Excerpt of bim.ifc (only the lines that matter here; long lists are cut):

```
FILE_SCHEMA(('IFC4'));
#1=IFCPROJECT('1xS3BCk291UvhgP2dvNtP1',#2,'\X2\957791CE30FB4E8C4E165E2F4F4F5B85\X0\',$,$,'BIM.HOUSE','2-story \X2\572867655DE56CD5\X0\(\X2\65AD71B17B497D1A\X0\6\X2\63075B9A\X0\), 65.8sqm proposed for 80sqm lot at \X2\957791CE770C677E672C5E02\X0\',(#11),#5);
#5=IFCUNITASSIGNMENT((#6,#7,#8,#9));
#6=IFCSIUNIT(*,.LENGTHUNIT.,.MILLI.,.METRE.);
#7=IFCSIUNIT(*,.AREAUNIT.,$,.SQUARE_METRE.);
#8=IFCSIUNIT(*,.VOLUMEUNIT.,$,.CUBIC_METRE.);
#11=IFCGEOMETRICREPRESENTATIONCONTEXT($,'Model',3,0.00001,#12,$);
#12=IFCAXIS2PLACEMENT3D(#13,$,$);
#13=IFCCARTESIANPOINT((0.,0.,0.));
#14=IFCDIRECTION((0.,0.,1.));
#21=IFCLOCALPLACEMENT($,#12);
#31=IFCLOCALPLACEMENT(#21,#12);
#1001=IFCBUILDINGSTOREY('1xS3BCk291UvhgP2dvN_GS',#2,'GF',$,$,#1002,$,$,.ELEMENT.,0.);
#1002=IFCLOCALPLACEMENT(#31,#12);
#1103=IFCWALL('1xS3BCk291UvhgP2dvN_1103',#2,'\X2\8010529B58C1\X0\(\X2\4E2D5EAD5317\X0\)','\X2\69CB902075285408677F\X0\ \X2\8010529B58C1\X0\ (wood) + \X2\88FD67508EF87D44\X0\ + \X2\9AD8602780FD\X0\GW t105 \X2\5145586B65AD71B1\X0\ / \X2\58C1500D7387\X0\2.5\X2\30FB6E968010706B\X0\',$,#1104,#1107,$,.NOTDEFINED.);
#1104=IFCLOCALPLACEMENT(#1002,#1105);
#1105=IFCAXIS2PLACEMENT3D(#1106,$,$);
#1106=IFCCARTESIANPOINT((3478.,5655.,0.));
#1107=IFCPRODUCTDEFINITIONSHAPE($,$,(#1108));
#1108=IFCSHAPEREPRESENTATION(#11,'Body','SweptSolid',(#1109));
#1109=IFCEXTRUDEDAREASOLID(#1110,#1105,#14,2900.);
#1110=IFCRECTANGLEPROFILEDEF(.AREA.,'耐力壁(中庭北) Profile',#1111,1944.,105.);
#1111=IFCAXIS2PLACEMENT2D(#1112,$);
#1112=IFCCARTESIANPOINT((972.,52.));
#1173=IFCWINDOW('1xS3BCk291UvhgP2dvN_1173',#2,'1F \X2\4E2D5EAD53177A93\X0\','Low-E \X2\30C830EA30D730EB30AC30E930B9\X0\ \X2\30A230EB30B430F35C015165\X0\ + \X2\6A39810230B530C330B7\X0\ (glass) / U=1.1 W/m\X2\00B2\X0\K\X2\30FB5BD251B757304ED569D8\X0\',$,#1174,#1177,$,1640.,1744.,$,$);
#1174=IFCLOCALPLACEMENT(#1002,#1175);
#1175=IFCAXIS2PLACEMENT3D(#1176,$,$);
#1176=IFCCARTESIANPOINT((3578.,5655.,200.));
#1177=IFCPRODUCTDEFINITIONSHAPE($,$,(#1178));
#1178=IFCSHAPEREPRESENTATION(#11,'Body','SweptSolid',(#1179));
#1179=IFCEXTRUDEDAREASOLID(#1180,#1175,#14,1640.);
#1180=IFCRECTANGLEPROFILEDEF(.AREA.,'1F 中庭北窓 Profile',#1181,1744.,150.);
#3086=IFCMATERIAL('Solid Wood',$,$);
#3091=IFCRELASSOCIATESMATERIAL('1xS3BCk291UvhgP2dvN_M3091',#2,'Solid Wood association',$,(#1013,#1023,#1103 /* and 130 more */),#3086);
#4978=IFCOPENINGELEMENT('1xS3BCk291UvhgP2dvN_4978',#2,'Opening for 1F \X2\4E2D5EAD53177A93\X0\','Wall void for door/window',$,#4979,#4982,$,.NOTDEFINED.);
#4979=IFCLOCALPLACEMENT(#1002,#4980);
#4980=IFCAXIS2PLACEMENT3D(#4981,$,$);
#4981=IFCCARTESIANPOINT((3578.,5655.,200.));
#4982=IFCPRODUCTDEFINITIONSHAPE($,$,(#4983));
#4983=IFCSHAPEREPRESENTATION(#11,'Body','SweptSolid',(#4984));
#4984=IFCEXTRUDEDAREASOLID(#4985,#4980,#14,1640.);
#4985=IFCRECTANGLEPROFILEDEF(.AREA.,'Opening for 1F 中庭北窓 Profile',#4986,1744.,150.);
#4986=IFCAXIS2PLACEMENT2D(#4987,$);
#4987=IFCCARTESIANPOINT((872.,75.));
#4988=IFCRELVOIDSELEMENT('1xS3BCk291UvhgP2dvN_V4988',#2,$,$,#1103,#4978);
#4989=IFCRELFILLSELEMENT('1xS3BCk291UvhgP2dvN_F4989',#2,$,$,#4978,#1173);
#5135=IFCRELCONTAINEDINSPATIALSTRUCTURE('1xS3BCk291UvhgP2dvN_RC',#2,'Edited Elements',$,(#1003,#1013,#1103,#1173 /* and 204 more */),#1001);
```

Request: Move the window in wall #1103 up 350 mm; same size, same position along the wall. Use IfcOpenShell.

```python
import numpy as np
import ifcopenshell
import ifcopenshell.api.geometry
import ifcopenshell.util.placement
import ifcopenshell.util.unit

model = ifcopenshell.open("bim.ifc")
unit_scale = ifcopenshell.util.unit.calculate_unit_scale(model)

window = model.by_id(1173)
opening = window.FillsVoids[0].RelatingOpeningElement
dz = 350.0

shift = np.array([0.0, 0.0, dz])
# The window is not placed relative to its opening, so move both.
for product in (opening, window):
    matrix = ifcopenshell.util.placement.get_local_placement(product.ObjectPlacement)
    matrix[:3, 3] += shift
    ifcopenshell.api.geometry.edit_object_placement(model, product=product, matrix=matrix, is_si=False)

print(f"moved by {dz * unit_scale:+.3f} m")

model.write("bim_rev.ifc")
```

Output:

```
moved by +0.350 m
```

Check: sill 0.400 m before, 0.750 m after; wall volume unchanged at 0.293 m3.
